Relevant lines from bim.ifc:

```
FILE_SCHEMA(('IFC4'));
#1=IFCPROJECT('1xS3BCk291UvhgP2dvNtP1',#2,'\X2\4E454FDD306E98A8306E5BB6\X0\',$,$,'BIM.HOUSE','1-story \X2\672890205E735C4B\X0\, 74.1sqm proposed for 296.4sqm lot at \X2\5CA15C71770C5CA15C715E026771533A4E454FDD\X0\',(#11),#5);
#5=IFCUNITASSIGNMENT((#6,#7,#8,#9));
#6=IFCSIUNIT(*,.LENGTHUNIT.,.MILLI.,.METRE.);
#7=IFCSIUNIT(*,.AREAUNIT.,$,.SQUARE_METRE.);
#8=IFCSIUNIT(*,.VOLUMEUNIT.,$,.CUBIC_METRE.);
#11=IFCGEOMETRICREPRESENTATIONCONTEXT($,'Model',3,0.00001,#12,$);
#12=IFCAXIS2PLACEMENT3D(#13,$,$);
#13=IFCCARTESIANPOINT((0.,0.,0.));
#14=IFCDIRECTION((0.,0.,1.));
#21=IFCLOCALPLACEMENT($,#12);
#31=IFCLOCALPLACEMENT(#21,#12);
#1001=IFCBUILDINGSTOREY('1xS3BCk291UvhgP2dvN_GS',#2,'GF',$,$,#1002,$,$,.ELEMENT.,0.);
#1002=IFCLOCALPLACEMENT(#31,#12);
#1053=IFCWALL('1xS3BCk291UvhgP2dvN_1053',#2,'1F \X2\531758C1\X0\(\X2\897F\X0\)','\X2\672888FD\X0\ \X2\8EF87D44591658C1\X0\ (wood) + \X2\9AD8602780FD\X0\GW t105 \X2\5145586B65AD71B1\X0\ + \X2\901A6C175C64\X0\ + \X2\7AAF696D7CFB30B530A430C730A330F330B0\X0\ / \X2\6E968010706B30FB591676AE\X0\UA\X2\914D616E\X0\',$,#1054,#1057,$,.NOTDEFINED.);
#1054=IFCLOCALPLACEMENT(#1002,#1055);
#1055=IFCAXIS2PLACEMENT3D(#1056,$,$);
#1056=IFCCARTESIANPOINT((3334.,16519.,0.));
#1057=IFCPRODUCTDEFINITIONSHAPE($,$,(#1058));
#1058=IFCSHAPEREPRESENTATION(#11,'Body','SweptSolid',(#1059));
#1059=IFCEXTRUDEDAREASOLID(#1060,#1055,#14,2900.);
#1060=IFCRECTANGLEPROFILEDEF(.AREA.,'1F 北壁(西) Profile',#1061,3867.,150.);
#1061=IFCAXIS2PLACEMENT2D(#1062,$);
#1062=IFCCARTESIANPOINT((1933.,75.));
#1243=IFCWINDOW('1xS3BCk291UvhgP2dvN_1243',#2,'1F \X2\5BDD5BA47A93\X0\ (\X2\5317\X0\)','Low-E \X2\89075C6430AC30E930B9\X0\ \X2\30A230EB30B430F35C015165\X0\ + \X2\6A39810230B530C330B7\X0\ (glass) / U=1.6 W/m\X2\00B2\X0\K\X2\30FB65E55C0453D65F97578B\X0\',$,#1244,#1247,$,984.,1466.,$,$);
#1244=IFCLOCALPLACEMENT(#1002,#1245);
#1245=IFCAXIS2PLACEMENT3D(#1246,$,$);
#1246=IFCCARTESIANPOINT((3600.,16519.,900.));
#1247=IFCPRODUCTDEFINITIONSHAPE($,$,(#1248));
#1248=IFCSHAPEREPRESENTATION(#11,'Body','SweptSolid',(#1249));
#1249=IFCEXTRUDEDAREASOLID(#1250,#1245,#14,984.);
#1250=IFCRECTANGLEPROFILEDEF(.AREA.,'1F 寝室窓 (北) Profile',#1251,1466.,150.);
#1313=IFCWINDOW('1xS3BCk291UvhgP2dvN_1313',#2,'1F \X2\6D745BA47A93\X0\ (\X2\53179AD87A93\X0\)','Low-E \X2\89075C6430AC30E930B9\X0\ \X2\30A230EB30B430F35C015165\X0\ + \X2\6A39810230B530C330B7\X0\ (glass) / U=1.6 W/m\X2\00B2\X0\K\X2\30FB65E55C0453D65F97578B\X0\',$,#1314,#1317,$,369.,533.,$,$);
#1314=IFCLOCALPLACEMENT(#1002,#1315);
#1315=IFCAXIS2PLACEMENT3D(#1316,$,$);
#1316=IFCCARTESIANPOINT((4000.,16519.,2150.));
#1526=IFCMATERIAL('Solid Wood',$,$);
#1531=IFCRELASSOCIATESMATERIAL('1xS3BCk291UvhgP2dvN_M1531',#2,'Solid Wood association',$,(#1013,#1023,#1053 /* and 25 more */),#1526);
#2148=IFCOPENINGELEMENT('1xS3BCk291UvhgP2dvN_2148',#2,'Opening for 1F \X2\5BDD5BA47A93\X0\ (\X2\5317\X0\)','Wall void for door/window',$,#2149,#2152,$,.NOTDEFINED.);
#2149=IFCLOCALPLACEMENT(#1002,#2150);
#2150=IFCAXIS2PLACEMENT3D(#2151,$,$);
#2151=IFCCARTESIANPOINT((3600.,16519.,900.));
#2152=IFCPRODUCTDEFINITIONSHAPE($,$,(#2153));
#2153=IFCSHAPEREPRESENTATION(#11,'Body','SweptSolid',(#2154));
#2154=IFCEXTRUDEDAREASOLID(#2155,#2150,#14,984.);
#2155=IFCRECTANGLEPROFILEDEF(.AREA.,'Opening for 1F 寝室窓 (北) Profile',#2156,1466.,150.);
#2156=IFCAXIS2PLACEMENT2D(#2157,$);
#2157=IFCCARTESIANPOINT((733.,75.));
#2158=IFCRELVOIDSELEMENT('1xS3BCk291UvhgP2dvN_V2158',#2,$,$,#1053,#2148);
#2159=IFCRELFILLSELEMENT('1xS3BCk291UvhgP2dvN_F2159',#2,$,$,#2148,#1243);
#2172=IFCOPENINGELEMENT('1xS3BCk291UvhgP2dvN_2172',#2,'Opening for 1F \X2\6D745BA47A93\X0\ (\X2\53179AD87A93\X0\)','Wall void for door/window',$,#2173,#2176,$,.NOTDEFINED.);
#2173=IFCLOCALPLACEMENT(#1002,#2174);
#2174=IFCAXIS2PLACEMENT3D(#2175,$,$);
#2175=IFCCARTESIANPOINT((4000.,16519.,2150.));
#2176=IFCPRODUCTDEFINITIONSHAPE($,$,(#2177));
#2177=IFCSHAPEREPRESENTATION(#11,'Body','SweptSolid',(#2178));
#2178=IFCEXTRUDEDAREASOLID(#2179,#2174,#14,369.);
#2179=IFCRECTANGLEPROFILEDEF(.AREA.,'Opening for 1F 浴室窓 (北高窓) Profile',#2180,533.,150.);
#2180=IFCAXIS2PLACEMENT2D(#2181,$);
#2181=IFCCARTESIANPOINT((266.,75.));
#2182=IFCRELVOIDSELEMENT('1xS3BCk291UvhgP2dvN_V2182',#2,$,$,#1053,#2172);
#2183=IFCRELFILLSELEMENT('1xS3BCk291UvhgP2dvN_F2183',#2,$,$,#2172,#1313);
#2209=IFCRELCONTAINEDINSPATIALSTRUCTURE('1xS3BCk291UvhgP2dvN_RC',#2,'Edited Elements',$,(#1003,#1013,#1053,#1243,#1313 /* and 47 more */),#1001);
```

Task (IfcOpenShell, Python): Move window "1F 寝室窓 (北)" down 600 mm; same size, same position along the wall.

```python
import numpy as np
import ifcopenshell
import ifcopenshell.api.geometry
import ifcopenshell.util.placement
import ifcopenshell.util.unit

model = ifcopenshell.open("bim.ifc")
unit_scale = ifcopenshell.util.unit.calculate_unit_scale(model)

window = model.by_guid("1xS3BCk291UvhgP2dvN_1243")
opening = window.FillsVoids[0].RelatingOpeningElement
dz = -0.6 / unit_scale

shift = np.array([0.0, 0.0, dz])
# The window is not placed relative to its opening, so move both.
for product in (opening, window):
    matrix = ifcopenshell.util.placement.get_local_placement(product.ObjectPlacement)
    matrix[:3, 3] += shift
    ifcopenshell.api.geometry.edit_object_placement(model, product=product, matrix=matrix, is_si=False)

print(f"moved by {dz * unit_scale:+.3f} m")

model.write("bim_rev.ifc")
```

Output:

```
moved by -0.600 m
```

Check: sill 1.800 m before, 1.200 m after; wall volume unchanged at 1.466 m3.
